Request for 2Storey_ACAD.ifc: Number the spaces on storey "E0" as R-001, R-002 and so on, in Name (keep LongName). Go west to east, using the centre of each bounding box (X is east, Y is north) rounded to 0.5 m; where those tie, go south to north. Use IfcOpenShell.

First a look at what the model holds.

```python
import ifcopenshell
import ifcopenshell.util.element
import ifcopenshell.util.placement

model = ifcopenshell.open("2Storey_ACAD.ifc")
print(model.schema)
storey = next(s for s in model.by_type("IfcBuildingStorey") if s.Name == "E0")
spaces = [e for e in ifcopenshell.util.element.get_decomposition(storey) if e.is_a("IfcSpace")]
for e in sorted(spaces, key=lambda e: e.id()):
    origin = ifcopenshell.util.placement.get_local_placement(e.ObjectPlacement)[:3, 3]
    print(e.id(), e.Name, e.LongName, origin.round(2) + 0.0, sep=" | ")
```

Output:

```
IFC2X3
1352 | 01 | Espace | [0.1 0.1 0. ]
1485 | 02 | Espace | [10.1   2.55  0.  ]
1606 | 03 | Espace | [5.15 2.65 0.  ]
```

```python
import ifcopenshell
import ifcopenshell.geom
import ifcopenshell.util.element
import ifcopenshell.util.shape

model = ifcopenshell.open("2Storey_ACAD.ifc")
settings = ifcopenshell.geom.settings()
settings.set("use-world-coords", True)


def centre(element):
    shape = ifcopenshell.geom.create_shape(settings, element)
    return ifcopenshell.util.shape.get_bbox_centroid(shape.geometry)


storey = next(s for s in model.by_type("IfcBuildingStorey") if s.Name == "E0")
spaces = [e for e in ifcopenshell.util.element.get_decomposition(storey) if e.is_a("IfcSpace")]

# Insertion points can sit at a corner or the storey origin, so sort by the geometry (in metres).
centres = {e: centre(e) for e in spaces}
spaces.sort(key=lambda e: (round(centres[e][0] / 0.5), centres[e][1]))

for i, e in enumerate(spaces, start=1):
    number = f"R-0{i:02d}"
    e.Name = number
    print(e.id(), number)

model.write("2Storey_ACAD_v2.ifc")
```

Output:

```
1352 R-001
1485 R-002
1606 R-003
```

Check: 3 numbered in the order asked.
